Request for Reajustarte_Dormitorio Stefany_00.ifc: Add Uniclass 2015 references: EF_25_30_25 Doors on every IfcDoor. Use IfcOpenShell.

First a look at what the model holds.

```python
import ifcopenshell

model = ifcopenshell.open("Reajustarte_Dormitorio Stefany_00.ifc")
print(model.schema)
print("classifications:", [c.Name for c in model.by_type("IfcClassification")])
for ifc_class in ("IfcDoor", "IfcRoof", "IfcStair", "IfcWall", "IfcWindow"):
    print(ifc_class, len(model.by_type(ifc_class)))
```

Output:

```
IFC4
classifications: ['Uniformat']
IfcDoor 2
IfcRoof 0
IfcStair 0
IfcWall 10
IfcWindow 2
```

```python
import ifcopenshell
import ifcopenshell.api.classification

model = ifcopenshell.open("Reajustarte_Dormitorio Stefany_00.ifc")

system = ifcopenshell.api.classification.add_classification(model, classification="Uniclass 2015")

codes = {
    "IfcDoor": ("EF_25_30_25", "Doors"),
}
for ifc_class, (code, name) in codes.items():
    products = model.by_type(ifc_class)
    ifcopenshell.api.classification.add_reference(
        model, products=products, classification=system, identification=code, name=name
    )
    print(code, len(products))

model.write("Reajustarte_Dormitorio Stefany_00_edited.ifc")
```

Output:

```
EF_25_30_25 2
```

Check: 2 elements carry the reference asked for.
